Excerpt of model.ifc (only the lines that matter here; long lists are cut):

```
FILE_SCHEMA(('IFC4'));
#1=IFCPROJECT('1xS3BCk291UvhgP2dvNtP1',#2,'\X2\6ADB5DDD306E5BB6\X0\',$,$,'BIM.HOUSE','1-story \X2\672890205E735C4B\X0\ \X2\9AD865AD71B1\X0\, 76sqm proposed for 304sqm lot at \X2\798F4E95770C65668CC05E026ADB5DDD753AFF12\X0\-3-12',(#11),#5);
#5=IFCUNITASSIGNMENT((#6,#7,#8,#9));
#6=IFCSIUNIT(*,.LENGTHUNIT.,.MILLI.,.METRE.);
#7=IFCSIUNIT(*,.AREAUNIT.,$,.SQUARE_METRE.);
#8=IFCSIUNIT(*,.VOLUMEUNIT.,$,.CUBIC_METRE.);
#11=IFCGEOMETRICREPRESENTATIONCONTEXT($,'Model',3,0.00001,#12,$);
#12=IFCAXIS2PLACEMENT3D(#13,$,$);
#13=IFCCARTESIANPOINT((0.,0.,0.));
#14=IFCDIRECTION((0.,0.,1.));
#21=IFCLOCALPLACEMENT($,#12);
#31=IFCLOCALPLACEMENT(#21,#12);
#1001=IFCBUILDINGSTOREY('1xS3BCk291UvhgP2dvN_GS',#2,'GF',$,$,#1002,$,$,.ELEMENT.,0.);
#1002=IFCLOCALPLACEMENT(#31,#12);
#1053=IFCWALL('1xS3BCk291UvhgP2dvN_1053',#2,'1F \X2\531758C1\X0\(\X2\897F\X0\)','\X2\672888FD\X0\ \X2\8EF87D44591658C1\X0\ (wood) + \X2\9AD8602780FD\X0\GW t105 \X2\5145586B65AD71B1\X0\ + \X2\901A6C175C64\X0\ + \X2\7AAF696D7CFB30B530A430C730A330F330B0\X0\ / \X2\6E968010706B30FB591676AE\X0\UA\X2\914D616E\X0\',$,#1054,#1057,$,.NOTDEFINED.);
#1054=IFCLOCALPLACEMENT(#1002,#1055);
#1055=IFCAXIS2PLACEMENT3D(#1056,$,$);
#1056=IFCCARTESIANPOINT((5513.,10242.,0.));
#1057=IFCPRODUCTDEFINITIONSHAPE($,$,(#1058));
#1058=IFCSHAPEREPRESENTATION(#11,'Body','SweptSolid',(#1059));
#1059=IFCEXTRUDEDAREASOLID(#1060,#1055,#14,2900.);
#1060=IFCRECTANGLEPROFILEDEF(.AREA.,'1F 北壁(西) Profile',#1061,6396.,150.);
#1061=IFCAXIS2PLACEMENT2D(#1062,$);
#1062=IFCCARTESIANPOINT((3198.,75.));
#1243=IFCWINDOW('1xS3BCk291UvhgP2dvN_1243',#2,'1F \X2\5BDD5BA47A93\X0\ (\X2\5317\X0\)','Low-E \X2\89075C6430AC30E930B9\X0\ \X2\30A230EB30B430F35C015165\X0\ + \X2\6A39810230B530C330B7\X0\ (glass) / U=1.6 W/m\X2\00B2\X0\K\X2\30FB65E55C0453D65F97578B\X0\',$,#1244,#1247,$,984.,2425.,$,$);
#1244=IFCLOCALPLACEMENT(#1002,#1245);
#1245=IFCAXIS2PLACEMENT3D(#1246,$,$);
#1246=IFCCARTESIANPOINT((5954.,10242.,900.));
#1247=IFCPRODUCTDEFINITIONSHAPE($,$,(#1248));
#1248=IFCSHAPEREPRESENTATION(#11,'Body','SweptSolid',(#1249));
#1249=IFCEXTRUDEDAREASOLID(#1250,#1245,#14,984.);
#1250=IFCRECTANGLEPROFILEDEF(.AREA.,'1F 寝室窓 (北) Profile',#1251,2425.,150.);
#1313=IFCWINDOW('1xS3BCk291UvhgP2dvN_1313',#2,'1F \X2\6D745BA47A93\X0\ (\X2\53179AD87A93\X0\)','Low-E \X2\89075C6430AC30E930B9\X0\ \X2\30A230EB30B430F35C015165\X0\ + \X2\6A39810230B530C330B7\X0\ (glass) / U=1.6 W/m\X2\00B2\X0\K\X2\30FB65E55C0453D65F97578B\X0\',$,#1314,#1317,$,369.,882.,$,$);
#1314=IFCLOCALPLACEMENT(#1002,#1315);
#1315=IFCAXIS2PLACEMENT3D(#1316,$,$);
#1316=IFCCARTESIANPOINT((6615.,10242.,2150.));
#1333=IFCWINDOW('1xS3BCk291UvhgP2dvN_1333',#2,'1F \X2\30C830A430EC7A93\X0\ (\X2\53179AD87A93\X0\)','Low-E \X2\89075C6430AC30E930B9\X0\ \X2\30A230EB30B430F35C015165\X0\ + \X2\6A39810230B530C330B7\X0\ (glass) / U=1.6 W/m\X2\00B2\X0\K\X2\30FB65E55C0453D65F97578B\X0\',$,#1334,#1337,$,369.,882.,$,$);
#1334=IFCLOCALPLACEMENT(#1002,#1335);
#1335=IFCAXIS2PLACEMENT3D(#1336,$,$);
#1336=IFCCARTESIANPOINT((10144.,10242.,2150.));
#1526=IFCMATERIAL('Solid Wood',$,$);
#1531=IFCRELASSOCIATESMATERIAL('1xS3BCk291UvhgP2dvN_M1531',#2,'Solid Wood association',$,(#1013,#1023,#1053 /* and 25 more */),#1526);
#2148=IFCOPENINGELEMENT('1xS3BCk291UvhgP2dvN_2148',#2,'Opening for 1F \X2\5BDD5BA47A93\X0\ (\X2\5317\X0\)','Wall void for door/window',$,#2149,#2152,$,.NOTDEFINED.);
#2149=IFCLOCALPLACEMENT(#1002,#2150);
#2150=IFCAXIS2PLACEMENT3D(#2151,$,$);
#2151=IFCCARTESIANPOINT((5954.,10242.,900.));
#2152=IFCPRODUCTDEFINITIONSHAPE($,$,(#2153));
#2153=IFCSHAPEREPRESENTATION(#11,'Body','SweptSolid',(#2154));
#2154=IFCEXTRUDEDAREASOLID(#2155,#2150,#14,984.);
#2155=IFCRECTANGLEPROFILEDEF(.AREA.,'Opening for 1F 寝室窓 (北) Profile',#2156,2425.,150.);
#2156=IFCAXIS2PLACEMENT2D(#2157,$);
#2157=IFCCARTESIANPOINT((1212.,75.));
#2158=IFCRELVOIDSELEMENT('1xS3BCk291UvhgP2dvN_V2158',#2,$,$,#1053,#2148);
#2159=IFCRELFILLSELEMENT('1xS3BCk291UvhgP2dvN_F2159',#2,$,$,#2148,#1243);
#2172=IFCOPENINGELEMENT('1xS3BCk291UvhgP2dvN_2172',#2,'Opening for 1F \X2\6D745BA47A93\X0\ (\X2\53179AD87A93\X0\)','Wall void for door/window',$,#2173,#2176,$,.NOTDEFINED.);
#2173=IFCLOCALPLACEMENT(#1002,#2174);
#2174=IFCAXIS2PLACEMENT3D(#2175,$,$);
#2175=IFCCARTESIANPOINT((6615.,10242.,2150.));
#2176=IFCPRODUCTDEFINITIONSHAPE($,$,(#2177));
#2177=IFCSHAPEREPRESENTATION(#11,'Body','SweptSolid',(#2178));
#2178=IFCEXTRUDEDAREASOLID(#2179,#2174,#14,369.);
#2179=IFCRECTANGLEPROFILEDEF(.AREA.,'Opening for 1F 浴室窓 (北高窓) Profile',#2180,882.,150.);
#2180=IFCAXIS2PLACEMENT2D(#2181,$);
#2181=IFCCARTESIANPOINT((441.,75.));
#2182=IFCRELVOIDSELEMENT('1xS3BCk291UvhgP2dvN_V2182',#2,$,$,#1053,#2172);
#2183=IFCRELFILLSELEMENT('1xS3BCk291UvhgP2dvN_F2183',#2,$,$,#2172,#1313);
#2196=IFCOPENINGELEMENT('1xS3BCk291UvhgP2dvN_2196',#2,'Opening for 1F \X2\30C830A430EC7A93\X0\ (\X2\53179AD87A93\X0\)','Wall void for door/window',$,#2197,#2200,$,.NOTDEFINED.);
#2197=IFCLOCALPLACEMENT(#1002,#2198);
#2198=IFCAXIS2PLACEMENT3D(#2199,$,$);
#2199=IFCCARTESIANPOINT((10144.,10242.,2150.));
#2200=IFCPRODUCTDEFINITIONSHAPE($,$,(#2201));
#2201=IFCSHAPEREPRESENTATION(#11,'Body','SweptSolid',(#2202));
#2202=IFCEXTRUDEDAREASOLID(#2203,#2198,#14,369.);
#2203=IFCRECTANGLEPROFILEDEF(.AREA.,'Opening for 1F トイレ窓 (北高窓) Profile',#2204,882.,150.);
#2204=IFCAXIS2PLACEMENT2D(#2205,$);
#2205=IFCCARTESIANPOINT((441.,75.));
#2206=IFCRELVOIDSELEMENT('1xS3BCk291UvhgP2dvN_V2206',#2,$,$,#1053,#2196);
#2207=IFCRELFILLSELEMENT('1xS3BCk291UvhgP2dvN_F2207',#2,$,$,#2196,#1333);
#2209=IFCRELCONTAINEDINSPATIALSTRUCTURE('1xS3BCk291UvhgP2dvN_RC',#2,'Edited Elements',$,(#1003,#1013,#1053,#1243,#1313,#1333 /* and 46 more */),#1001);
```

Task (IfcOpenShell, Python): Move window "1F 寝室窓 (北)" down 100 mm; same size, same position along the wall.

```python
import numpy as np
import ifcopenshell
import ifcopenshell.api.geometry
import ifcopenshell.util.placement
import ifcopenshell.util.unit

model = ifcopenshell.open("model.ifc")
unit_scale = ifcopenshell.util.unit.calculate_unit_scale(model)

window = model.by_guid("1xS3BCk291UvhgP2dvN_1243")
opening = window.FillsVoids[0].RelatingOpeningElement
dz = -100.0

shift = np.array([0.0, 0.0, dz])
# The window is not placed relative to its opening, so move both.
for product in (opening, window):
    matrix = ifcopenshell.util.placement.get_local_placement(product.ObjectPlacement)
    matrix[:3, 3] += shift
    ifcopenshell.api.geometry.edit_object_placement(model, product=product, matrix=matrix, is_si=False)

print(f"moved by {dz * unit_scale:+.3f} m")

model.write("model_rev.ifc")
```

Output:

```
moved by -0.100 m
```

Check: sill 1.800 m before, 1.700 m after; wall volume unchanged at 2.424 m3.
